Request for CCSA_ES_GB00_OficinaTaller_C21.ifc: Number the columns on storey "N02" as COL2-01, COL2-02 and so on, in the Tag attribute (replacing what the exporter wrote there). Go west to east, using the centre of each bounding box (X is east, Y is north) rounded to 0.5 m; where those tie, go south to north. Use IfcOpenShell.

First a look at what the model holds.

```python
import ifcopenshell
import ifcopenshell.util.element
import ifcopenshell.util.placement

model = ifcopenshell.open("CCSA_ES_GB00_OficinaTaller_C21.ifc")
print(model.schema)
storey = next(s for s in model.by_type("IfcBuildingStorey") if s.Name == "N02")
columns = [e for e in ifcopenshell.util.element.get_decomposition(storey) if e.is_a("IfcColumn")]
for e in sorted(columns, key=lambda e: e.id()):
    origin = ifcopenshell.util.placement.get_local_placement(e.ObjectPlacement)[:3, 3]
    print(e.id(), e.Tag, e.Name, origin.round(2) + 0.0, sep=" | ")
```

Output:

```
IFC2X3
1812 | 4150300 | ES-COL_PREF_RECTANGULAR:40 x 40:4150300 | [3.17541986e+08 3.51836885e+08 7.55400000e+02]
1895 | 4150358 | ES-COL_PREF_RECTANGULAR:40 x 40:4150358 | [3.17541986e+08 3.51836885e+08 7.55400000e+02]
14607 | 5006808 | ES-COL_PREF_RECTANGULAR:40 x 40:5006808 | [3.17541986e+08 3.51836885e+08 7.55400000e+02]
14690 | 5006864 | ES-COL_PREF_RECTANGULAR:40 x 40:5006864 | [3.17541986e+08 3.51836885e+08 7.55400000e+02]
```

```python
import ifcopenshell
import ifcopenshell.geom
import ifcopenshell.util.element
import ifcopenshell.util.shape

model = ifcopenshell.open("CCSA_ES_GB00_OficinaTaller_C21.ifc")
settings = ifcopenshell.geom.settings()
settings.set("use-world-coords", True)


def centre(element):
    shape = ifcopenshell.geom.create_shape(settings, element)
    return ifcopenshell.util.shape.get_bbox_centroid(shape.geometry)


storey = next(s for s in model.by_type("IfcBuildingStorey") if s.Name == "N02")
columns = [e for e in ifcopenshell.util.element.get_decomposition(storey) if e.is_a("IfcColumn")]

# Insertion points can sit at a corner or the storey origin, so sort by the geometry (in metres).
centres = {e: centre(e) for e in columns}
columns.sort(key=lambda e: (round(centres[e][0] / 0.5), centres[e][1]))

for i, e in enumerate(columns, start=1):
    number = f"COL2-{i:02d}"
    e.Tag = number
    print(e.id(), number)

model.write("CCSA_ES_GB00_OficinaTaller_C21_edited.ifc")
```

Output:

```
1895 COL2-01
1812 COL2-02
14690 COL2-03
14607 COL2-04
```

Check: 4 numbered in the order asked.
